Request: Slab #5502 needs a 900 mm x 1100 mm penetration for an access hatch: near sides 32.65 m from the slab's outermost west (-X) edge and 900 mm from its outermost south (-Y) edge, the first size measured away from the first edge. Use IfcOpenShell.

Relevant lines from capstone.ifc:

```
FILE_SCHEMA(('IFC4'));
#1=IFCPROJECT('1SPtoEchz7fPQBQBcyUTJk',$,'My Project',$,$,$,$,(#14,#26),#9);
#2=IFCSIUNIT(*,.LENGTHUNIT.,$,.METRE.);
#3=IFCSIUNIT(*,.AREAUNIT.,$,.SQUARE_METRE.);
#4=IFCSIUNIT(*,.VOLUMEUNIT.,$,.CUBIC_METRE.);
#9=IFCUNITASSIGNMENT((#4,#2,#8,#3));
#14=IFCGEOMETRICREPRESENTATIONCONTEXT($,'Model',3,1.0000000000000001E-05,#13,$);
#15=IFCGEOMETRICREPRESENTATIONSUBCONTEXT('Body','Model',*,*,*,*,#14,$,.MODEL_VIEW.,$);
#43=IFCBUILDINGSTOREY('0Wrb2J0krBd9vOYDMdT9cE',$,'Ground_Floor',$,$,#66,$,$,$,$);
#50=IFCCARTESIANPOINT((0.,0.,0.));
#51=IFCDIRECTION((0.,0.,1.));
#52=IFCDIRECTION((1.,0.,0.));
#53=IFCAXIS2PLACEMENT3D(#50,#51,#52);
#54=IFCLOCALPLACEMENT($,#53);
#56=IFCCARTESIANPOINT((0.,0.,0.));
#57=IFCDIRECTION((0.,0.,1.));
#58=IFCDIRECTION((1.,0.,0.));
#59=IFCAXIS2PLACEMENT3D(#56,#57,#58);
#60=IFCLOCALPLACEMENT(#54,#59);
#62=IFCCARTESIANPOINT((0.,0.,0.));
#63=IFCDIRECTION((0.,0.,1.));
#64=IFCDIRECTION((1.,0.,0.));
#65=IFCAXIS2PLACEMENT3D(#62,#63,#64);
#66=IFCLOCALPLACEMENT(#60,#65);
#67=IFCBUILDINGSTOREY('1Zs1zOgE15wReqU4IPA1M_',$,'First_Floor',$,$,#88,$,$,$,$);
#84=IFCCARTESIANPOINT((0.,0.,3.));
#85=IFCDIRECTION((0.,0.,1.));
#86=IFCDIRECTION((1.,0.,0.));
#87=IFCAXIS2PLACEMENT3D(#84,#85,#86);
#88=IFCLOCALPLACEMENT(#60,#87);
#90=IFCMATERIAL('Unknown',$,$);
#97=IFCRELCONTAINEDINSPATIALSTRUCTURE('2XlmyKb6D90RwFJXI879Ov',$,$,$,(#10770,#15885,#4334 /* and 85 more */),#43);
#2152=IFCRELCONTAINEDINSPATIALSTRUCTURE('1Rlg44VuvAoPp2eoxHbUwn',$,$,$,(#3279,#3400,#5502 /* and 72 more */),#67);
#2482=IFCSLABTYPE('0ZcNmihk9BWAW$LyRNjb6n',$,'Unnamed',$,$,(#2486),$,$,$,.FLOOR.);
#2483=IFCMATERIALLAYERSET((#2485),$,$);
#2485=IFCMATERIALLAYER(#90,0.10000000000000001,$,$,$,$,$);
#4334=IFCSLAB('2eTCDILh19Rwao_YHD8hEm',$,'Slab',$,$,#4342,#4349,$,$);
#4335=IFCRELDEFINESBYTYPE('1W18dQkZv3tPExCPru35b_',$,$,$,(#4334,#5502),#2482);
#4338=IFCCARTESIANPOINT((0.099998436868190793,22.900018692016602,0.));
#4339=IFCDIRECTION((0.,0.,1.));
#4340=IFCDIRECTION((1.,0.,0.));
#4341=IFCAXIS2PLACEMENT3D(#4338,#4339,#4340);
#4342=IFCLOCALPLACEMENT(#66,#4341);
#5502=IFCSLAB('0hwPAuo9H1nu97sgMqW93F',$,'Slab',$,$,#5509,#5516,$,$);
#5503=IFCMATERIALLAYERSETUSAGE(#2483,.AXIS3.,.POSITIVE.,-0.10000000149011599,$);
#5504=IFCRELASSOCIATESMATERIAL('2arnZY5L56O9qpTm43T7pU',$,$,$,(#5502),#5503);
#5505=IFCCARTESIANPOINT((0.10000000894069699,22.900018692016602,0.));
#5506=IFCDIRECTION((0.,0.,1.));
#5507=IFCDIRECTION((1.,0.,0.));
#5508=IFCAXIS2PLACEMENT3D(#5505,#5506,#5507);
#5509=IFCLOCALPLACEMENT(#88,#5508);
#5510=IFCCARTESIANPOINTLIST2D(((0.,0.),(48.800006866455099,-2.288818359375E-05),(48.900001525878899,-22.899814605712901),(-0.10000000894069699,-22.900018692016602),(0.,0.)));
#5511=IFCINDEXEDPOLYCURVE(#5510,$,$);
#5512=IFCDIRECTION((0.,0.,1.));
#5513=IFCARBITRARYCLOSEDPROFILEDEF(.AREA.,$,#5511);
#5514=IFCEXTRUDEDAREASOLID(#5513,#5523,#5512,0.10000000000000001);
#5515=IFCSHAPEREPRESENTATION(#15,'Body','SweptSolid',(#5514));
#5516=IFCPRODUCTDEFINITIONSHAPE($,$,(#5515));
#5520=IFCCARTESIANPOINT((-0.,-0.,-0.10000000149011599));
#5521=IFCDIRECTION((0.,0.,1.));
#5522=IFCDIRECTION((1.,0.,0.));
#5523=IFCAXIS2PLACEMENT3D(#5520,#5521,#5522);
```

```python
import numpy as np
import ifcopenshell
import ifcopenshell.api.feature
import ifcopenshell.api.geometry
import ifcopenshell.api.root
import ifcopenshell.geom
import ifcopenshell.util.placement
import ifcopenshell.util.representation
import ifcopenshell.util.shape
import ifcopenshell.util.unit

model = ifcopenshell.open("capstone.ifc")
unit_scale = ifcopenshell.util.unit.calculate_unit_scale(model)
settings = ifcopenshell.geom.settings()


def volume(element):
    """Net volume in cubic metres, openings subtracted."""
    shape = ifcopenshell.geom.create_shape(settings, element)
    return ifcopenshell.util.shape.get_volume(shape.geometry)


slab = model.by_id(5502)
before = volume(slab)

# Extent in the slab's own axes, in metres. The edges named are its -X and -Y sides.
slab_shape = ifcopenshell.geom.create_shape(settings, slab)
vertices = ifcopenshell.util.shape.get_vertices(slab_shape.geometry)
x_min, y_min, bottom = vertices.min(axis=0)
top = vertices[:, 2].max()

opening = ifcopenshell.api.root.create_entity(model, ifc_class="IfcOpeningElement", name="Access hatch opening", predefined_type="OPENING")
context = ifcopenshell.util.representation.get_context(model, "Model", "Body", "MODEL_VIEW")
width, depth = 0.9, 1.1
outline = [(0.0, 0.0), (width, 0.0), (width, depth), (0.0, depth), (0.0, 0.0)]
# Overshoot both faces by 50 mm so the cut is clean.
shape = ifcopenshell.api.geometry.add_slab_representation(
    model, context=context, depth=top - bottom + 0.1, polyline=outline
)
ifcopenshell.api.geometry.assign_representation(model, product=opening, representation=shape)

matrix = ifcopenshell.util.placement.get_local_placement(slab.ObjectPlacement)
matrix[:, 3] = matrix @ np.append(np.array([x_min + 32.65, y_min + 0.9, bottom - 0.05]) / unit_scale, 1.0)
ifcopenshell.api.geometry.edit_object_placement(model, product=opening, matrix=matrix, is_si=False)
ifcopenshell.api.feature.add_feature(model, feature=opening, element=slab)

after = volume(slab)

print(f"slab volume {before:.3f} -> {after:.3f} m3")

model.write("capstone_v2.ifc")
```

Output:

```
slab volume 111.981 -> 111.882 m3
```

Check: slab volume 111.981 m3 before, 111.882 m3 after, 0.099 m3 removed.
